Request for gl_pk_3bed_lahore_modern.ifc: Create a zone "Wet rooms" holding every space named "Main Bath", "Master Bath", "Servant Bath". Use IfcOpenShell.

First a look at what the model holds.

```python
import ifcopenshell

model = ifcopenshell.open("gl_pk_3bed_lahore_modern.ifc")
print(model.schema)
seen = {}
for space in model.by_type("IfcSpace"):
    seen[space.LongName] = seen.get(space.LongName, 0) + 1
for name, count in sorted(seen.items(), key=str):
    print(count, "x", name)
print("zones:", [z.Name for z in model.by_type("IfcZone")][:20])
```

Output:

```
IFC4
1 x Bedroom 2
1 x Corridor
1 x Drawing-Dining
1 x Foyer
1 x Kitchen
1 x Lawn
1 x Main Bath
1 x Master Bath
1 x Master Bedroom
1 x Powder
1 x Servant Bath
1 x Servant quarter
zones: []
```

```python
import ifcopenshell
import ifcopenshell.api.group
import ifcopenshell.api.root

model = ifcopenshell.open("gl_pk_3bed_lahore_modern.ifc")

names = {"Main Bath", "Master Bath", "Servant Bath"}
spaces = [s for s in model.by_type("IfcSpace") if s.LongName in names]

zone = ifcopenshell.api.root.create_entity(model, ifc_class="IfcZone", name="Wet rooms")
ifcopenshell.api.group.assign_group(model, products=spaces, group=zone)
print(len(spaces), "spaces in", zone.Name)

model.write("gl_pk_3bed_lahore_modern_v2.ifc")
```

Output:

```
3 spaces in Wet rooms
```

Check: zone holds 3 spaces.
